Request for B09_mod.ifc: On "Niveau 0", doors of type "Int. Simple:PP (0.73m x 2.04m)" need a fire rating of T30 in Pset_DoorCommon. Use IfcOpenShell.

First a look at what the model holds.

```python
import ifcopenshell
import ifcopenshell.util.element

model = ifcopenshell.open("B09_mod.ifc")
print(model.schema)
storey = next(s for s in model.by_type("IfcBuildingStorey") if s.Name == "Niveau 0")
doors = [e for e in ifcopenshell.util.element.get_decomposition(storey) if e.is_a("IfcDoor")]
seen = {}
for e in doors:
    element_type = ifcopenshell.util.element.get_type(e)
    key = (element_type.Name if element_type != e and element_type else None, ifcopenshell.util.element.get_pset(e, "Pset_DoorCommon", "FireRating"))
    seen[key] = seen.get(key, 0) + 1
for (name, value), count in sorted(seen.items(), key=str):
    print(count, "x", name, "|", value)
```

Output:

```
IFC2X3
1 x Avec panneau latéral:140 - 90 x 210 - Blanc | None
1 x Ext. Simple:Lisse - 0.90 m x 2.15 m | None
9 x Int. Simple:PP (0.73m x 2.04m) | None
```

```python
import ifcopenshell
import ifcopenshell.api.pset
import ifcopenshell.util.element

model = ifcopenshell.open("B09_mod.ifc")

storey = next(s for s in model.by_type("IfcBuildingStorey") if s.Name == "Niveau 0")
doors = [e for e in ifcopenshell.util.element.get_decomposition(storey) if e.is_a("IfcDoor")]

count = 0
for e in doors:
    element_type = ifcopenshell.util.element.get_type(e)
    if element_type in (None, e) or element_type.Name != "Int. Simple:PP (0.73m x 2.04m)":
        continue
    # add_pset returns the element's existing set when there is one.
    pset = ifcopenshell.api.pset.add_pset(model, product=e, name="Pset_DoorCommon")
    ifcopenshell.api.pset.edit_pset(model, pset=pset, properties={"FireRating": "T30"})
    count += 1

print(count, "doors updated")

model.write("B09_mod_v2.ifc")
```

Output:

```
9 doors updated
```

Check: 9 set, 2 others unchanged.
